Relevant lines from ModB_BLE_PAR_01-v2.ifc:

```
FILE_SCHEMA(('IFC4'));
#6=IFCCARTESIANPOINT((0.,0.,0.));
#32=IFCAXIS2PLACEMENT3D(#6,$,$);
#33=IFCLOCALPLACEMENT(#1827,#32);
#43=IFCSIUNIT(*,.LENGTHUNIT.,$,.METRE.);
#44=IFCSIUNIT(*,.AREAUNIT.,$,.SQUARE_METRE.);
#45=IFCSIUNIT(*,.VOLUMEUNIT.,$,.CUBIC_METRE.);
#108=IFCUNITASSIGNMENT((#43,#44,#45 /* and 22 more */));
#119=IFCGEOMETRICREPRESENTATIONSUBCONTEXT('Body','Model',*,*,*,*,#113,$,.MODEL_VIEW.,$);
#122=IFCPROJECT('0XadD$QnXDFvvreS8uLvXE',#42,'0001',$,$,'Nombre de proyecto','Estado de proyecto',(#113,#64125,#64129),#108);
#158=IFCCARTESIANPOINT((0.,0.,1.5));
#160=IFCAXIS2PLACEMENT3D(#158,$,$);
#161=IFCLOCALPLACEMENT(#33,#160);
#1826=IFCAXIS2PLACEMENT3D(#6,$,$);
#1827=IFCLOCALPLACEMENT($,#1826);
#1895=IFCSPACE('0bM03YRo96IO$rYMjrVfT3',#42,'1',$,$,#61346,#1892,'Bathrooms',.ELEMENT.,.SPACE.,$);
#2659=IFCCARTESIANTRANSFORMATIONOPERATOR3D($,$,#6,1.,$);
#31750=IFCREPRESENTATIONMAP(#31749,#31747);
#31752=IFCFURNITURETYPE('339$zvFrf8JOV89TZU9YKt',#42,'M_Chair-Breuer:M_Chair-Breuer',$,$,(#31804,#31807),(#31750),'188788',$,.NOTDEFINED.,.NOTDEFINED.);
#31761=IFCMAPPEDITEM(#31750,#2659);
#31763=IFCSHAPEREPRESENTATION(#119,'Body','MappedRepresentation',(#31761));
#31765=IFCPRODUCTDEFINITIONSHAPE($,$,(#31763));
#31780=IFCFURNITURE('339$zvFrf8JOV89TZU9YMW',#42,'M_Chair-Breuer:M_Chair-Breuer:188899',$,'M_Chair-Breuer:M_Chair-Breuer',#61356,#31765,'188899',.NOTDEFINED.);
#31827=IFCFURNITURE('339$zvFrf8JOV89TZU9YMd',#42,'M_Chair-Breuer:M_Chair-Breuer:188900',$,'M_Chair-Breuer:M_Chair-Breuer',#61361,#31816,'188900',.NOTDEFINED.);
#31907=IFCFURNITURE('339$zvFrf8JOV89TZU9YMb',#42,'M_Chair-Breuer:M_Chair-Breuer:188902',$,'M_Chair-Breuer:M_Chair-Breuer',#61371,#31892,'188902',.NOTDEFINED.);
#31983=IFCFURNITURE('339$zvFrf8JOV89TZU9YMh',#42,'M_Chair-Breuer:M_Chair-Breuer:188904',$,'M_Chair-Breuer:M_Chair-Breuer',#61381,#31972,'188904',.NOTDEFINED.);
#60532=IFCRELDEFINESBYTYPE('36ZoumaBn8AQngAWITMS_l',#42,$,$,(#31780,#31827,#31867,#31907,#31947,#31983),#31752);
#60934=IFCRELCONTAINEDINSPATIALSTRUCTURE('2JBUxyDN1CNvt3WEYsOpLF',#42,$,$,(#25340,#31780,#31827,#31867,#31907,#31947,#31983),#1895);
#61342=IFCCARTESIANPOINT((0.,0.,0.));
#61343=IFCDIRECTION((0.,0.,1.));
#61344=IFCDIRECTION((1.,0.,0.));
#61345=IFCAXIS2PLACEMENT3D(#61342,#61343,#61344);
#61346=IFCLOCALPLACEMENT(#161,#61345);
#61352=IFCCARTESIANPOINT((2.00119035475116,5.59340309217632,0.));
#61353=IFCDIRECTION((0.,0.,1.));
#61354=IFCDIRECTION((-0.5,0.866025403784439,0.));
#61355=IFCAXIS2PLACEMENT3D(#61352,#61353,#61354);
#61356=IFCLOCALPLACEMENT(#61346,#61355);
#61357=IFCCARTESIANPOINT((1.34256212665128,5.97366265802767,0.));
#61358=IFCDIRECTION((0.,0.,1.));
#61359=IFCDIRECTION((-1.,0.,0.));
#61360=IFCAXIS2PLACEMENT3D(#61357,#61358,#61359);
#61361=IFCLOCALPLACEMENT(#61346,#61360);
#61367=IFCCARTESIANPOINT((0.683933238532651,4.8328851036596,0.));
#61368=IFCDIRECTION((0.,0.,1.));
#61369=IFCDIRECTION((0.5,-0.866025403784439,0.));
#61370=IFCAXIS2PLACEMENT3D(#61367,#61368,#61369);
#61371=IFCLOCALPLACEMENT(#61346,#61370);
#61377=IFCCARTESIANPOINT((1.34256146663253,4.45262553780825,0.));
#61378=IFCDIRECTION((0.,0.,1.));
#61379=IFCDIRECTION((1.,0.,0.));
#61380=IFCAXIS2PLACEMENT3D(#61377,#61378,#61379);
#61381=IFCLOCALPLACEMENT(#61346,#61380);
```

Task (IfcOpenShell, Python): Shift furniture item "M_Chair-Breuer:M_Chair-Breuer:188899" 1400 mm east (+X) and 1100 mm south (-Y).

```python
import ifcopenshell
import ifcopenshell.api.geometry
import ifcopenshell.util.placement
import ifcopenshell.util.unit

model = ifcopenshell.open("ModB_BLE_PAR_01-v2.ifc")
unit_scale = ifcopenshell.util.unit.calculate_unit_scale(model)

item = model.by_id(31780)
matrix = ifcopenshell.util.placement.get_local_placement(item.ObjectPlacement)
matrix[0, 3] += 1.4 / unit_scale
matrix[1, 3] -= 1.1 / unit_scale
ifcopenshell.api.geometry.edit_object_placement(model, product=item, matrix=matrix, is_si=False)

print(ifcopenshell.util.placement.get_local_placement(item.ObjectPlacement).round(3) + 0.0)

model.write("ModB_BLE_PAR_01-v2_v2.ifc")
```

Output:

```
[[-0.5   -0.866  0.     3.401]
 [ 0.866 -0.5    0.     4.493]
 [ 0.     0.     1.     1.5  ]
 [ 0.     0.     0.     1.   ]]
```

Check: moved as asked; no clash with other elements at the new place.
